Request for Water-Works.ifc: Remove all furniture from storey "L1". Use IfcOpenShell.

First a look at what the model holds.

```python
import ifcopenshell
import ifcopenshell.util.element

model = ifcopenshell.open("Water-Works.ifc")
print(model.schema)
storey = next(s for s in model.by_type("IfcBuildingStorey") if s.Name == "L1")
furniture = [e for e in ifcopenshell.util.element.get_decomposition(storey) if e.is_a("IfcFurnishingElement")]
seen = {}
for e in furniture:
    element_type = ifcopenshell.util.element.get_type(e)
    name = element_type.Name if element_type not in (None, e) else None
    seen[name] = seen.get(name, 0) + 1
for name, count in sorted(seen.items(), key=str):
    print(count, "x", name)
```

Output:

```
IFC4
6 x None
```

```python
import ifcopenshell
import ifcopenshell.api.root
import ifcopenshell.util.element

model = ifcopenshell.open("Water-Works.ifc")

storey = next(s for s in model.by_type("IfcBuildingStorey") if s.Name == "L1")
furniture = [e for e in ifcopenshell.util.element.get_decomposition(storey) if e.is_a("IfcFurnishingElement")]

for e in furniture:
    ifcopenshell.api.root.remove_product(model, product=e)
print(len(furniture), "removed")

model.write("Water-Works_edited.ifc")
```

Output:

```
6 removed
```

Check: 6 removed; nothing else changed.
